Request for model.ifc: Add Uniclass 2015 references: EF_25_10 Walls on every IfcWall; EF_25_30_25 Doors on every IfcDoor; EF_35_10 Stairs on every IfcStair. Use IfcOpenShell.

First a look at what the model holds.

```python
import ifcopenshell

model = ifcopenshell.open("model.ifc")
print(model.schema)
print("classifications:", [c.Name for c in model.by_type("IfcClassification")])
for ifc_class in ("IfcDoor", "IfcRoof", "IfcStair", "IfcWall", "IfcWindow"):
    print(ifc_class, len(model.by_type(ifc_class)))
```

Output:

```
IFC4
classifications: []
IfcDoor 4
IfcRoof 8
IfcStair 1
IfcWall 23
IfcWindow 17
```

```python
import ifcopenshell
import ifcopenshell.api.classification

model = ifcopenshell.open("model.ifc")

system = ifcopenshell.api.classification.add_classification(model, classification="Uniclass 2015")

codes = {
    "IfcWall": ("EF_25_10", "Walls"),
    "IfcDoor": ("EF_25_30_25", "Doors"),
    "IfcStair": ("EF_35_10", "Stairs"),
}
for ifc_class, (code, name) in codes.items():
    products = model.by_type(ifc_class)
    ifcopenshell.api.classification.add_reference(
        model, products=products, classification=system, identification=code, name=name
    )
    print(code, len(products))

model.write("model_edited.ifc")
```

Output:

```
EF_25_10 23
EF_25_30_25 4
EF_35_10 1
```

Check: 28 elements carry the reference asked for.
